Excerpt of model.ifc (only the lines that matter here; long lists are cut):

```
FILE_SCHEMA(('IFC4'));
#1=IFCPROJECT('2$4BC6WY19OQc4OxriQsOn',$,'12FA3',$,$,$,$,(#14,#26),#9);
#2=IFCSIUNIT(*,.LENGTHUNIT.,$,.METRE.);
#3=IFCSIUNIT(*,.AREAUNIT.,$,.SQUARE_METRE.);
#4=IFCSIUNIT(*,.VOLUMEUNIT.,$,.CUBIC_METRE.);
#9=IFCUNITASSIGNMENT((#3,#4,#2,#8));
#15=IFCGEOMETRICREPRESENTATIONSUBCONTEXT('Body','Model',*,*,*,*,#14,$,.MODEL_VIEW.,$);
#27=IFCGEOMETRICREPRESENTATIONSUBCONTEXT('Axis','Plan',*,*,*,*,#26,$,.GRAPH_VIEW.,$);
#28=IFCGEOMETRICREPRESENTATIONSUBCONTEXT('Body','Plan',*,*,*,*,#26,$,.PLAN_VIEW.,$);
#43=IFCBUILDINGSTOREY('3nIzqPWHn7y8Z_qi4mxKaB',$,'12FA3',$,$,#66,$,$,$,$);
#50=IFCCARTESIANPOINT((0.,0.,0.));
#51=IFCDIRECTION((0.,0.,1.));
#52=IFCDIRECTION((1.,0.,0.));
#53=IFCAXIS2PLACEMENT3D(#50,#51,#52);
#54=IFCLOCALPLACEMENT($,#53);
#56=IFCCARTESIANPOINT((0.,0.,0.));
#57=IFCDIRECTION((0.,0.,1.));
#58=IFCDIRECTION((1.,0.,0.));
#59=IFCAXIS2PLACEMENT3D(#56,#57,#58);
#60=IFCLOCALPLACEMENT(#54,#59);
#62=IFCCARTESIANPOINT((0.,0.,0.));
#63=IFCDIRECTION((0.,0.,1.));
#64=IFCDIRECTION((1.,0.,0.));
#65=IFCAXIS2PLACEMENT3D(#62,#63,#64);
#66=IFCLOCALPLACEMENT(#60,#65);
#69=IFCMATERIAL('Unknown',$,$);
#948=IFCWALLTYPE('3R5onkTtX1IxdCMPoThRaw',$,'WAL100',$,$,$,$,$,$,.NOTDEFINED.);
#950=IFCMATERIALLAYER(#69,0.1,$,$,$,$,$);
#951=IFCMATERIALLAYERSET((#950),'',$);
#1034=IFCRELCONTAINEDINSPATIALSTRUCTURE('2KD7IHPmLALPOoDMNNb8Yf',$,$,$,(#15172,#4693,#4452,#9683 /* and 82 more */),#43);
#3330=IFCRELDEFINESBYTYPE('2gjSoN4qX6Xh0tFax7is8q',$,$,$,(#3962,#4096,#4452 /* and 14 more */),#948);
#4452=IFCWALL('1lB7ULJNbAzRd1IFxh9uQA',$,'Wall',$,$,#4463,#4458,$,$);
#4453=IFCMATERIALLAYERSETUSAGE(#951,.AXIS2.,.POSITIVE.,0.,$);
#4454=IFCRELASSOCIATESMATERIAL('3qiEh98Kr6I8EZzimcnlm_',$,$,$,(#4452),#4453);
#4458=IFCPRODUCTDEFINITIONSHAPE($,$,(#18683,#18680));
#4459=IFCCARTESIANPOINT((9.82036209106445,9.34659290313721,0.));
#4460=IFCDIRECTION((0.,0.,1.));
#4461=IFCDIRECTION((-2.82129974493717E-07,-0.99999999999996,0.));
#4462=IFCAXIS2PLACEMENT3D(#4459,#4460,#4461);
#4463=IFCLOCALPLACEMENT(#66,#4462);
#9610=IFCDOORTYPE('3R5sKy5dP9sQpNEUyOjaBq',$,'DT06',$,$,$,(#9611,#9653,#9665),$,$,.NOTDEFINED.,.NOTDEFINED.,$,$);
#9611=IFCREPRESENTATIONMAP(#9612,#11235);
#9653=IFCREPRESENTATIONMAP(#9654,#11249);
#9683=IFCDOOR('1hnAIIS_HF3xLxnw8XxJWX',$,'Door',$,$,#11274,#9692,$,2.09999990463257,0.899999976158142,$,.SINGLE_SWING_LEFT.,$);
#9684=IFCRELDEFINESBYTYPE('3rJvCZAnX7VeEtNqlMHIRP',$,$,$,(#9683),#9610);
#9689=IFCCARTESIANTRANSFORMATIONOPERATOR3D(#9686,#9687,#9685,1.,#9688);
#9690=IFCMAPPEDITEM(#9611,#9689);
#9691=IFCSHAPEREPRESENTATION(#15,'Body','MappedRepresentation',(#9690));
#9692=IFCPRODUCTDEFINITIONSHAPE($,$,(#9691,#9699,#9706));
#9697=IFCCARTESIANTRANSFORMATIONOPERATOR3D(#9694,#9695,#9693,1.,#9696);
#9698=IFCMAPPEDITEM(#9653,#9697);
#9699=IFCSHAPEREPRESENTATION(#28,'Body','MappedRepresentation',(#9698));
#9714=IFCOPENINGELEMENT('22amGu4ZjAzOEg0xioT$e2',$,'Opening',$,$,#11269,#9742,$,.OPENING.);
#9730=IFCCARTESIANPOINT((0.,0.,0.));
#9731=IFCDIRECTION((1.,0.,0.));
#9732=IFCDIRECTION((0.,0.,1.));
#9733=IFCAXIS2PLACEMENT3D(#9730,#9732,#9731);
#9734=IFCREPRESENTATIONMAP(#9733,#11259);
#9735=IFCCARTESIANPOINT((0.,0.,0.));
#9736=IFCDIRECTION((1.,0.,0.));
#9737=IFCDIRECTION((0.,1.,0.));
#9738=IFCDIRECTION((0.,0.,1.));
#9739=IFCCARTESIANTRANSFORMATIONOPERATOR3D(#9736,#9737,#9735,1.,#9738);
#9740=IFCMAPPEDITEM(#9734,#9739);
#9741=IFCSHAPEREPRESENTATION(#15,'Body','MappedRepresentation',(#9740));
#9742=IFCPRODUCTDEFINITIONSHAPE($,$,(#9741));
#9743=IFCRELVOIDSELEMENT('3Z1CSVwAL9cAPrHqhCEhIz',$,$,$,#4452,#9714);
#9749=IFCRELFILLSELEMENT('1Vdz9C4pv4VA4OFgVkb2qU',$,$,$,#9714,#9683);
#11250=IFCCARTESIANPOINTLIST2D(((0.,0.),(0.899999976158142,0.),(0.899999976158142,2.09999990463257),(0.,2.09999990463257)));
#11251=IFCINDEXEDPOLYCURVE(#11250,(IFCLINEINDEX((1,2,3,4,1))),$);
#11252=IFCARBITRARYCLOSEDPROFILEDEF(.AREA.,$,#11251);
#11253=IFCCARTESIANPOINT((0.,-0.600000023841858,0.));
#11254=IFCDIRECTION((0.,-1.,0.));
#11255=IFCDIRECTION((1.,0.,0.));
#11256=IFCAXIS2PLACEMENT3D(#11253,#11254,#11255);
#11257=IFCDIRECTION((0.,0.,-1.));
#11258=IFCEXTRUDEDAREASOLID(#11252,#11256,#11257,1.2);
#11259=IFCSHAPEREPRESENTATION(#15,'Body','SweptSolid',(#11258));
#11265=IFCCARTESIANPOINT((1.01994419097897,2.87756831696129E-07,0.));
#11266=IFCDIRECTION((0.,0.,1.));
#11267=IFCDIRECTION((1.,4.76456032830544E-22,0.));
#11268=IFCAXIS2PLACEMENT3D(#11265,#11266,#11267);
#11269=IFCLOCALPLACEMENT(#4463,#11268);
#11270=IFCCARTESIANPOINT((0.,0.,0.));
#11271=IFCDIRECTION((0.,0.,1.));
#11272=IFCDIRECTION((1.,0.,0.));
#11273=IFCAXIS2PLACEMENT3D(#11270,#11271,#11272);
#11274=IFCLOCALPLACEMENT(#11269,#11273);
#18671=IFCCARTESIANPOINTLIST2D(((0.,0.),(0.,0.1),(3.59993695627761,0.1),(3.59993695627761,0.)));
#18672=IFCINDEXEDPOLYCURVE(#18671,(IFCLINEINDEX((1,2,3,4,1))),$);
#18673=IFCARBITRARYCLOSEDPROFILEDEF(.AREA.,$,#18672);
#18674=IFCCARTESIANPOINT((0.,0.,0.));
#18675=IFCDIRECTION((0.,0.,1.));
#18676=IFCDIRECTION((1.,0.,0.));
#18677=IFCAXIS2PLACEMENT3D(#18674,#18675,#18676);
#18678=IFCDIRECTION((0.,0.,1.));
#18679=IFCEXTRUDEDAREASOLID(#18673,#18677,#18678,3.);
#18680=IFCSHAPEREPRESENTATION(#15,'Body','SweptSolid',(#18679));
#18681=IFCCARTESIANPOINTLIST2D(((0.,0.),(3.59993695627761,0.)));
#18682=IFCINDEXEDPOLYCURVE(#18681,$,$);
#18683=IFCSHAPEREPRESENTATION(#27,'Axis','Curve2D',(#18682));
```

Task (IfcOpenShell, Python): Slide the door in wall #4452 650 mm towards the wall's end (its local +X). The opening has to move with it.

```python
import ifcopenshell
import ifcopenshell.api.geometry
import ifcopenshell.util.placement
import ifcopenshell.util.unit

model = ifcopenshell.open("model.ifc")
unit_scale = ifcopenshell.util.unit.calculate_unit_scale(model)

door = model.by_guid("1hnAIIS_HF3xLxnw8XxJWX")
opening = door.FillsVoids[0].RelatingOpeningElement
wall = opening.VoidsElements[0].RelatingBuildingElement

wall_matrix = ifcopenshell.util.placement.get_local_placement(wall.ObjectPlacement)
shift = wall_matrix[:3, 0] * 0.65 / unit_scale
before = ifcopenshell.util.placement.get_local_placement(door.ObjectPlacement)[:3, 3].copy()

# The door is placed relative to its opening, so it follows when the opening moves.
matrix = ifcopenshell.util.placement.get_local_placement(opening.ObjectPlacement)
matrix[:3, 3] += shift
ifcopenshell.api.geometry.edit_object_placement(
    model, product=opening, matrix=matrix, is_si=False, should_transform_children=True
)

after = ifcopenshell.util.placement.get_local_placement(door.ObjectPlacement)[:3, 3]
print("door moved by", (after - before).round(3) + 0.0)

model.write("model_updated.ifc")
```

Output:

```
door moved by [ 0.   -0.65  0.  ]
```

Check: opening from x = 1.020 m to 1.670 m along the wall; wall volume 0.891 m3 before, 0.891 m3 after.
